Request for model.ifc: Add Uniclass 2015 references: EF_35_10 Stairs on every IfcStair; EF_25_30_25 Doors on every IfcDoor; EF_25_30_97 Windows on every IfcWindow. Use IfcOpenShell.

First a look at what the model holds.

```python
import ifcopenshell

model = ifcopenshell.open("model.ifc")
print(model.schema)
print("classifications:", [c.Name for c in model.by_type("IfcClassification")])
for ifc_class in ("IfcDoor", "IfcRoof", "IfcStair", "IfcWall", "IfcWindow"):
    print(ifc_class, len(model.by_type(ifc_class)))
```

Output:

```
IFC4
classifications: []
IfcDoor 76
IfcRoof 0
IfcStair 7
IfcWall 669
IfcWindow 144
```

```python
import ifcopenshell
import ifcopenshell.api.classification

model = ifcopenshell.open("model.ifc")

system = ifcopenshell.api.classification.add_classification(model, classification="Uniclass 2015")

codes = {
    "IfcStair": ("EF_35_10", "Stairs"),
    "IfcDoor": ("EF_25_30_25", "Doors"),
    "IfcWindow": ("EF_25_30_97", "Windows"),
}
for ifc_class, (code, name) in codes.items():
    products = model.by_type(ifc_class)
    ifcopenshell.api.classification.add_reference(
        model, products=products, classification=system, identification=code, name=name
    )
    print(code, len(products))

model.write("model_rev.ifc")
```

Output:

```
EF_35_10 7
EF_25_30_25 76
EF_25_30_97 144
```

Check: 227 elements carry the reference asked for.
